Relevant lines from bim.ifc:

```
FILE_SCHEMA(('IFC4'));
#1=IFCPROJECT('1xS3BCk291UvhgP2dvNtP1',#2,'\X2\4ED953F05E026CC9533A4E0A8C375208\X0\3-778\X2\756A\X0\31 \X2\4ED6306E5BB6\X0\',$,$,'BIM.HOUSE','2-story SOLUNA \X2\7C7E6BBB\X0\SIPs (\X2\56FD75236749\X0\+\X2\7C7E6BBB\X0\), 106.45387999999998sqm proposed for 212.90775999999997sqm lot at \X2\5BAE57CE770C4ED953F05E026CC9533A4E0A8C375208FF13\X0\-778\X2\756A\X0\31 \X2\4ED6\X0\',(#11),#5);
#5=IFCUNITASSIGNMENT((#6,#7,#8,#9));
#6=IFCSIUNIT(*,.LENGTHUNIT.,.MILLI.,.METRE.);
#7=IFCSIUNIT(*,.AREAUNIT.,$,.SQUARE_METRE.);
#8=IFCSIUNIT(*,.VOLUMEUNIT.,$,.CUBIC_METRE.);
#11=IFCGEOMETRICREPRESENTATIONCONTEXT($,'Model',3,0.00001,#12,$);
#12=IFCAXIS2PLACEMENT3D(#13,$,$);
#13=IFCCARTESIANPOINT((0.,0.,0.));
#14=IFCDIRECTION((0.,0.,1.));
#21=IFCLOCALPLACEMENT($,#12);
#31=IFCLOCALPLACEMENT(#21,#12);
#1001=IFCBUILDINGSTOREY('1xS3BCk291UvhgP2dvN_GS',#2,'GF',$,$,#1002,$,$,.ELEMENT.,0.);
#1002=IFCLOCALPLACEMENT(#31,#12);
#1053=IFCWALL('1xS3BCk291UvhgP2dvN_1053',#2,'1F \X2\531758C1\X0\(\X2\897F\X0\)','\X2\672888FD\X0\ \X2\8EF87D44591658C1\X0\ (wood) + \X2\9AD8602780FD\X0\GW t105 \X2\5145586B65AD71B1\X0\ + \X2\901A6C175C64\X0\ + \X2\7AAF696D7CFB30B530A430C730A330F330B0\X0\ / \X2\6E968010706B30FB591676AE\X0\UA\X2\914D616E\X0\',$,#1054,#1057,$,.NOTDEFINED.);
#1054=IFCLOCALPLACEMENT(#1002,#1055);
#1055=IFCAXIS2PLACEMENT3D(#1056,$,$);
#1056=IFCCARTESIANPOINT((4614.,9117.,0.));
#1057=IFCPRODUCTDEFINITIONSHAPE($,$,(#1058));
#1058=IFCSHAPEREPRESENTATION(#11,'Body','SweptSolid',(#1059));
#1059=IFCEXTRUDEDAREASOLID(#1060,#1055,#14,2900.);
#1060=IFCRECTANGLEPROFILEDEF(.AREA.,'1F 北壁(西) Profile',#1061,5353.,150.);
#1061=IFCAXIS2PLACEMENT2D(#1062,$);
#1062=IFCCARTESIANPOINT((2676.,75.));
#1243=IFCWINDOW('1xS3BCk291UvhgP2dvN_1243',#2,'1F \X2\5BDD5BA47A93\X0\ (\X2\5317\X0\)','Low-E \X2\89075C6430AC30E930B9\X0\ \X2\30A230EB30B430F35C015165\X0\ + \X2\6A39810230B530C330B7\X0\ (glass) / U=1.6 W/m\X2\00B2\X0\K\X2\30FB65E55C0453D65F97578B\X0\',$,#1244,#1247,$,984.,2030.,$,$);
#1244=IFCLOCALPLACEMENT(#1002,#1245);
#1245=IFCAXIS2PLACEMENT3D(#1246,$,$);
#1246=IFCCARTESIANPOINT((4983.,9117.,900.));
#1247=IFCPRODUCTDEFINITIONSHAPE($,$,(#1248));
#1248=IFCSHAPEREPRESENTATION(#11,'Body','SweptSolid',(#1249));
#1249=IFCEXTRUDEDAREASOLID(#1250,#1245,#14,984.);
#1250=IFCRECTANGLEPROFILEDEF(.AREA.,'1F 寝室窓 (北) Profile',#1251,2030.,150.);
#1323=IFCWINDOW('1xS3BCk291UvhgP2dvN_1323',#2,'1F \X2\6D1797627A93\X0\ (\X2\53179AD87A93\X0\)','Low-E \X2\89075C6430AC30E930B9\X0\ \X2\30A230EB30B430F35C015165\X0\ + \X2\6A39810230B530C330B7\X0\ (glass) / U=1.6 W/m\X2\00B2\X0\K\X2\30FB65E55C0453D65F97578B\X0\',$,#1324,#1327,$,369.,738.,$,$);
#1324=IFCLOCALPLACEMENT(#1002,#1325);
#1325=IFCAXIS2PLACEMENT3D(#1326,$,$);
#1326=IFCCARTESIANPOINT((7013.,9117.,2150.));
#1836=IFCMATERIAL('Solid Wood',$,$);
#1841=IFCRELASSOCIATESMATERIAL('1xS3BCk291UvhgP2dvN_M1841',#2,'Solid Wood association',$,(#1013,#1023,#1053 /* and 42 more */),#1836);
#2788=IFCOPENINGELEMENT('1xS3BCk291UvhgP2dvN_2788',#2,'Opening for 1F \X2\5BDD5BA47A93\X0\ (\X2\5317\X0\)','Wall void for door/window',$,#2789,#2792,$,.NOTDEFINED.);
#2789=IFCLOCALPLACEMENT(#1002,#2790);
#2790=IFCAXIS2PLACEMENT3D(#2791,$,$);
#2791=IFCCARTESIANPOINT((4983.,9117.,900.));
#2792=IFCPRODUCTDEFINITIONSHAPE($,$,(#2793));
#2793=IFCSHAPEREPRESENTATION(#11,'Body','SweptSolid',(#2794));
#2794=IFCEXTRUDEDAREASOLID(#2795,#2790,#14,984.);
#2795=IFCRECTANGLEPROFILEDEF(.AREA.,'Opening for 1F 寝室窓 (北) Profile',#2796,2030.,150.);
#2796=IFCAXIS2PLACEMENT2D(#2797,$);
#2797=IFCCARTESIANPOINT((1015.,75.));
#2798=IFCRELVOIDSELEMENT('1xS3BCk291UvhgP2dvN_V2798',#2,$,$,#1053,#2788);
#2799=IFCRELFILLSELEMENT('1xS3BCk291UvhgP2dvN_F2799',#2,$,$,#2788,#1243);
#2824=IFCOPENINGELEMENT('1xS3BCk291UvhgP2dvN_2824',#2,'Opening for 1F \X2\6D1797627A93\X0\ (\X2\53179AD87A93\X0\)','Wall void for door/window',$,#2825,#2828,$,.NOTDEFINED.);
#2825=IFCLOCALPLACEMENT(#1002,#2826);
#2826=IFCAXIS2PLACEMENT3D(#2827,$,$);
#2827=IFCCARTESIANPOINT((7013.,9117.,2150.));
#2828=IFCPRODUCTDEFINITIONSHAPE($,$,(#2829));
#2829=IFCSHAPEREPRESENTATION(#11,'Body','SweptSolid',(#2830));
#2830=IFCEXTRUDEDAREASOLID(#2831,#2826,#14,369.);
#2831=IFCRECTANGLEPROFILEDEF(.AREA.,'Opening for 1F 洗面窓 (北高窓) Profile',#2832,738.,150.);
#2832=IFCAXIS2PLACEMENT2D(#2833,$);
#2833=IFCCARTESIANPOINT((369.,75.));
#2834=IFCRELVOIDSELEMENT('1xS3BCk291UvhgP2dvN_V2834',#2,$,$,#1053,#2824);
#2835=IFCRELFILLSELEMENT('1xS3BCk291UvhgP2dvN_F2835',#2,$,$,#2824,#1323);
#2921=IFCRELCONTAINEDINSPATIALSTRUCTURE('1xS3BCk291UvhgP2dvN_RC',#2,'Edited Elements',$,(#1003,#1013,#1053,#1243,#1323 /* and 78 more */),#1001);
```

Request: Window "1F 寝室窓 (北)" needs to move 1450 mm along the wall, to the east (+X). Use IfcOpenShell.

```python
import ifcopenshell
import ifcopenshell.api.geometry
import ifcopenshell.util.placement

model = ifcopenshell.open("bim.ifc")

window = model.by_guid("1xS3BCk291UvhgP2dvN_1243")
opening = window.FillsVoids[0].RelatingOpeningElement
wall = opening.VoidsElements[0].RelatingBuildingElement

wall_matrix = ifcopenshell.util.placement.get_local_placement(wall.ObjectPlacement)
shift = wall_matrix[:3, 0] * 1450.0
before = ifcopenshell.util.placement.get_local_placement(window.ObjectPlacement)[:3, 3].copy()

# The window is not placed relative to its opening, so move both.
for product in (opening, window):
    matrix = ifcopenshell.util.placement.get_local_placement(product.ObjectPlacement)
    matrix[:3, 3] += shift
    ifcopenshell.api.geometry.edit_object_placement(model, product=product, matrix=matrix, is_si=False)

after = ifcopenshell.util.placement.get_local_placement(window.ObjectPlacement)[:3, 3]
print("window moved by", (after - before).round(3) + 0.0)

model.write("bim_edited.ifc")
```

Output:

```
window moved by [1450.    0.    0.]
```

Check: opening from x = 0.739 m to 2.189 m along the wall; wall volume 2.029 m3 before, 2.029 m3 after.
